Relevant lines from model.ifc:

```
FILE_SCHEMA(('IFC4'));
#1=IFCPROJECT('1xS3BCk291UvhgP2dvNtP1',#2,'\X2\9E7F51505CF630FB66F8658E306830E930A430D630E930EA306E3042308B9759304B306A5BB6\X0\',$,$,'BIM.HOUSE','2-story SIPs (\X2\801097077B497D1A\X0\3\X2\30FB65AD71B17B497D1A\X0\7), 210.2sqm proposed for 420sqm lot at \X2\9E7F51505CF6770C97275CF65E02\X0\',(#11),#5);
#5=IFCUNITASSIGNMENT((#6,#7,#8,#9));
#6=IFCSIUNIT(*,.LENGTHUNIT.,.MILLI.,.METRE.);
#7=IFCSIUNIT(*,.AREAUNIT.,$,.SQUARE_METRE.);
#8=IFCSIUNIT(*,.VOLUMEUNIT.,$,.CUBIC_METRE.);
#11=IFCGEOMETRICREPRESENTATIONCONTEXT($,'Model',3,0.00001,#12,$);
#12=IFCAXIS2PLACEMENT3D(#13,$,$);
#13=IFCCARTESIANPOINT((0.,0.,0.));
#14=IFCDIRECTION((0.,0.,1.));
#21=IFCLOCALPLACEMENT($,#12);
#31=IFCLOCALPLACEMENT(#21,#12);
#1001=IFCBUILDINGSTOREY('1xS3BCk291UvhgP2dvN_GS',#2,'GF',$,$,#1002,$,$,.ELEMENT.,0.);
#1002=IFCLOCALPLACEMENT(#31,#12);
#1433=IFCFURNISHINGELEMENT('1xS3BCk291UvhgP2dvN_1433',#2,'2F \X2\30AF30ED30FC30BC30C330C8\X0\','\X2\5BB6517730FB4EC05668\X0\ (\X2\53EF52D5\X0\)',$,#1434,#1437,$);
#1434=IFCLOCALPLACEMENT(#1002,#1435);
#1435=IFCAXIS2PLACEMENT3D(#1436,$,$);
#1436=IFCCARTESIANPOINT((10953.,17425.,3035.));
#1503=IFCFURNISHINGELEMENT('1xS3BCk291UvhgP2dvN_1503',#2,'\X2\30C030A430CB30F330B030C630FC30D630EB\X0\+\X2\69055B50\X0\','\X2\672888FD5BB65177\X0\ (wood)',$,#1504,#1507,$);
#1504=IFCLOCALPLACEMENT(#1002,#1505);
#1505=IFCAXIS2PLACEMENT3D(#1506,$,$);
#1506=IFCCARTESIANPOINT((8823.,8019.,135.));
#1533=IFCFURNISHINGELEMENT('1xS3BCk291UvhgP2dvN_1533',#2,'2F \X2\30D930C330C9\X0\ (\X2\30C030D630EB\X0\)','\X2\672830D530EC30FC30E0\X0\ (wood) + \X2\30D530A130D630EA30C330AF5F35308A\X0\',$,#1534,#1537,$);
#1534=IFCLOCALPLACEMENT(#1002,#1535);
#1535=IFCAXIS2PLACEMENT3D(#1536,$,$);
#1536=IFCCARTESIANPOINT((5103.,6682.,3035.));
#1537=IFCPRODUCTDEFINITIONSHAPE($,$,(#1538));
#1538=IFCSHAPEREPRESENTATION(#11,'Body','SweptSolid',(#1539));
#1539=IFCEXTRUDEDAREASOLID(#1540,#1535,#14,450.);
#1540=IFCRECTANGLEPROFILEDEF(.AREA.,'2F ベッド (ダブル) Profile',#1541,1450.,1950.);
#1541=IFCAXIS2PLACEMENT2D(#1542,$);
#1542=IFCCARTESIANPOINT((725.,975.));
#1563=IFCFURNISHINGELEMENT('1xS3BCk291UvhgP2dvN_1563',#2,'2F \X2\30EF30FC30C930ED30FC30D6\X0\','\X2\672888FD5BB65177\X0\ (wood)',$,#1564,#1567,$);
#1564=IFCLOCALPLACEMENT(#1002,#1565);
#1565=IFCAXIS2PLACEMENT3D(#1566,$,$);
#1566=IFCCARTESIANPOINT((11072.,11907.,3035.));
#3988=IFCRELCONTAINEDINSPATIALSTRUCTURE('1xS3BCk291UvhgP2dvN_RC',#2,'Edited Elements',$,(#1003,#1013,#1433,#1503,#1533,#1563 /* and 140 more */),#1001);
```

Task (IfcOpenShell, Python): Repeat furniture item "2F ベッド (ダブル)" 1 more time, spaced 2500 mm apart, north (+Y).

```python
import numpy as np
import ifcopenshell
import ifcopenshell.api.geometry
import ifcopenshell.api.root
import ifcopenshell.util.element
import ifcopenshell.util.placement

model = ifcopenshell.open("model.ifc")


def reuse_history(source, copy):
    """copy_class also copies each property set's owner history, people and application; keep the originals."""
    for rel in copy.IsDefinedBy:
        if rel.is_a("IfcRelDefinesByProperties") and (history := rel.RelatingPropertyDefinition.OwnerHistory):
            rel.RelatingPropertyDefinition.OwnerHistory = source.OwnerHistory
            ifcopenshell.util.element.remove_deep2(model, history)


source = model.by_id(1533)
base = ifcopenshell.util.placement.get_local_placement(source.ObjectPlacement)
step = np.array([0.0, 1.0, 0.0]) * 2500.0

for i in range(1, 2):
    copy = ifcopenshell.api.root.copy_class(model, product=source)
    copy.Representation = ifcopenshell.util.element.copy_deep(
        model, source.Representation, exclude=["IfcGeometricRepresentationContext", "IfcRepresentationMap"]
    )
    reuse_history(source, copy)
    matrix = base.copy()
    matrix[:3, 3] += i * step
    print("added at", matrix[:3, 3].round(3) + 0.0)
    ifcopenshell.api.geometry.edit_object_placement(model, product=copy, matrix=matrix, is_si=False)

model.write("model_updated.ifc")
```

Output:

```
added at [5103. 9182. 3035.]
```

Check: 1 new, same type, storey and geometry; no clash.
